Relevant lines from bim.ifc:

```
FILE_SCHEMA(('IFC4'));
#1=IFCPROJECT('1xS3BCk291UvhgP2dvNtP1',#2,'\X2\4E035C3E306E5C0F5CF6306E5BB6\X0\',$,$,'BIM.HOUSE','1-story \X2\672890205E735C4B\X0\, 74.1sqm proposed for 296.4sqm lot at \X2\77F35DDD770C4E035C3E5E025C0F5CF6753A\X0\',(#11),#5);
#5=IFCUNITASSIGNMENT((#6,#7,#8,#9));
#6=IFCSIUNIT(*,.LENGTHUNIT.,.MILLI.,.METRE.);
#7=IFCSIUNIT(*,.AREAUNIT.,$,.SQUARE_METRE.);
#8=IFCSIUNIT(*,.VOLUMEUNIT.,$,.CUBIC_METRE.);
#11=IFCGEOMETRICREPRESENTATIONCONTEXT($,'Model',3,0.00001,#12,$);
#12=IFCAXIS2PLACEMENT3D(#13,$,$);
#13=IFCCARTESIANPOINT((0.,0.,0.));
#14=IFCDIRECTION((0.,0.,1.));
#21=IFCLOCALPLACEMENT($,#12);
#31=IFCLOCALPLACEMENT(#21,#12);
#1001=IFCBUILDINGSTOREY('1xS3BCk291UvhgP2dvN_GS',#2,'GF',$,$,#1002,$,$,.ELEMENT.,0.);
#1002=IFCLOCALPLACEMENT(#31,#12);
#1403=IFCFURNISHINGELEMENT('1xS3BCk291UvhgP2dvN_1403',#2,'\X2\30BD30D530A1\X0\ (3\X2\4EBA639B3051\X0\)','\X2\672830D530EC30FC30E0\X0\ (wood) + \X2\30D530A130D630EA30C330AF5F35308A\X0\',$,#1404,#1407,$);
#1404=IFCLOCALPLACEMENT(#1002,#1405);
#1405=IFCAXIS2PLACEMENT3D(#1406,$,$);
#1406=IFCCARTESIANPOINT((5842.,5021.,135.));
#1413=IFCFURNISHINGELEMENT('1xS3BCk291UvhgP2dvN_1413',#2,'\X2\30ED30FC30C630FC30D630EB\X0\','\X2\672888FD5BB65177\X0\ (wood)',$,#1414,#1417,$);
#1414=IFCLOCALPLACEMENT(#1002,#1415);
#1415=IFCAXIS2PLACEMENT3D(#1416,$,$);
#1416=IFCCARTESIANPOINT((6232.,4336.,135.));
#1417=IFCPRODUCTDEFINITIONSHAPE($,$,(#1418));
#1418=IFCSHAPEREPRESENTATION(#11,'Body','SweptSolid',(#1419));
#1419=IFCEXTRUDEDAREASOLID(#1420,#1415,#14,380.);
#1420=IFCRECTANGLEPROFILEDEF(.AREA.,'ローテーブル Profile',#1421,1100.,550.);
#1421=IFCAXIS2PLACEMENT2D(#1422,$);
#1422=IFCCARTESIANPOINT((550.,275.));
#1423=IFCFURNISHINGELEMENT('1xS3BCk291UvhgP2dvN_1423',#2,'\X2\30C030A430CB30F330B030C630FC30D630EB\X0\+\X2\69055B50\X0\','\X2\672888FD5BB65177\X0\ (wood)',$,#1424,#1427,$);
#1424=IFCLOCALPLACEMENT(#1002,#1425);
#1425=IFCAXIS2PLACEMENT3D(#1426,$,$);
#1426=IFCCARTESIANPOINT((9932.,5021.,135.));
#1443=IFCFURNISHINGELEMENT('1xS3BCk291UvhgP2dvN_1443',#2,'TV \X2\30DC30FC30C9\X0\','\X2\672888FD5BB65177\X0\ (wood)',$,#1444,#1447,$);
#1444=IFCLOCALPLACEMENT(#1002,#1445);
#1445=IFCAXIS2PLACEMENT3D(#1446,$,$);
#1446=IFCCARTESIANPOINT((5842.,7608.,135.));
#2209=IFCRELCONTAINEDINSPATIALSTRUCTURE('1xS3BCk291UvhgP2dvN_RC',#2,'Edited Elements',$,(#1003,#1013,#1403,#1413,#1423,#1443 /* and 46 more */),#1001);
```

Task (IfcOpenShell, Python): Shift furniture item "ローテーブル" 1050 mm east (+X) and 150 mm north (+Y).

```python
import ifcopenshell
import ifcopenshell.api.geometry
import ifcopenshell.util.placement
import ifcopenshell.util.unit

model = ifcopenshell.open("bim.ifc")
unit_scale = ifcopenshell.util.unit.calculate_unit_scale(model)

item = model.by_guid("1xS3BCk291UvhgP2dvN_1413")
matrix = ifcopenshell.util.placement.get_local_placement(item.ObjectPlacement)
matrix[0, 3] += 1.05 / unit_scale
matrix[1, 3] += 0.15 / unit_scale
ifcopenshell.api.geometry.edit_object_placement(model, product=item, matrix=matrix, is_si=False)

print(ifcopenshell.util.placement.get_local_placement(item.ObjectPlacement).round(3) + 0.0)

model.write("bim_updated.ifc")
```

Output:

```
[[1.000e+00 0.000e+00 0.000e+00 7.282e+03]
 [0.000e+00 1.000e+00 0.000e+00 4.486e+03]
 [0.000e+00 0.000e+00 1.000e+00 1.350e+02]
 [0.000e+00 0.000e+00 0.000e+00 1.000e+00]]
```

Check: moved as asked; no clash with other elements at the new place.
